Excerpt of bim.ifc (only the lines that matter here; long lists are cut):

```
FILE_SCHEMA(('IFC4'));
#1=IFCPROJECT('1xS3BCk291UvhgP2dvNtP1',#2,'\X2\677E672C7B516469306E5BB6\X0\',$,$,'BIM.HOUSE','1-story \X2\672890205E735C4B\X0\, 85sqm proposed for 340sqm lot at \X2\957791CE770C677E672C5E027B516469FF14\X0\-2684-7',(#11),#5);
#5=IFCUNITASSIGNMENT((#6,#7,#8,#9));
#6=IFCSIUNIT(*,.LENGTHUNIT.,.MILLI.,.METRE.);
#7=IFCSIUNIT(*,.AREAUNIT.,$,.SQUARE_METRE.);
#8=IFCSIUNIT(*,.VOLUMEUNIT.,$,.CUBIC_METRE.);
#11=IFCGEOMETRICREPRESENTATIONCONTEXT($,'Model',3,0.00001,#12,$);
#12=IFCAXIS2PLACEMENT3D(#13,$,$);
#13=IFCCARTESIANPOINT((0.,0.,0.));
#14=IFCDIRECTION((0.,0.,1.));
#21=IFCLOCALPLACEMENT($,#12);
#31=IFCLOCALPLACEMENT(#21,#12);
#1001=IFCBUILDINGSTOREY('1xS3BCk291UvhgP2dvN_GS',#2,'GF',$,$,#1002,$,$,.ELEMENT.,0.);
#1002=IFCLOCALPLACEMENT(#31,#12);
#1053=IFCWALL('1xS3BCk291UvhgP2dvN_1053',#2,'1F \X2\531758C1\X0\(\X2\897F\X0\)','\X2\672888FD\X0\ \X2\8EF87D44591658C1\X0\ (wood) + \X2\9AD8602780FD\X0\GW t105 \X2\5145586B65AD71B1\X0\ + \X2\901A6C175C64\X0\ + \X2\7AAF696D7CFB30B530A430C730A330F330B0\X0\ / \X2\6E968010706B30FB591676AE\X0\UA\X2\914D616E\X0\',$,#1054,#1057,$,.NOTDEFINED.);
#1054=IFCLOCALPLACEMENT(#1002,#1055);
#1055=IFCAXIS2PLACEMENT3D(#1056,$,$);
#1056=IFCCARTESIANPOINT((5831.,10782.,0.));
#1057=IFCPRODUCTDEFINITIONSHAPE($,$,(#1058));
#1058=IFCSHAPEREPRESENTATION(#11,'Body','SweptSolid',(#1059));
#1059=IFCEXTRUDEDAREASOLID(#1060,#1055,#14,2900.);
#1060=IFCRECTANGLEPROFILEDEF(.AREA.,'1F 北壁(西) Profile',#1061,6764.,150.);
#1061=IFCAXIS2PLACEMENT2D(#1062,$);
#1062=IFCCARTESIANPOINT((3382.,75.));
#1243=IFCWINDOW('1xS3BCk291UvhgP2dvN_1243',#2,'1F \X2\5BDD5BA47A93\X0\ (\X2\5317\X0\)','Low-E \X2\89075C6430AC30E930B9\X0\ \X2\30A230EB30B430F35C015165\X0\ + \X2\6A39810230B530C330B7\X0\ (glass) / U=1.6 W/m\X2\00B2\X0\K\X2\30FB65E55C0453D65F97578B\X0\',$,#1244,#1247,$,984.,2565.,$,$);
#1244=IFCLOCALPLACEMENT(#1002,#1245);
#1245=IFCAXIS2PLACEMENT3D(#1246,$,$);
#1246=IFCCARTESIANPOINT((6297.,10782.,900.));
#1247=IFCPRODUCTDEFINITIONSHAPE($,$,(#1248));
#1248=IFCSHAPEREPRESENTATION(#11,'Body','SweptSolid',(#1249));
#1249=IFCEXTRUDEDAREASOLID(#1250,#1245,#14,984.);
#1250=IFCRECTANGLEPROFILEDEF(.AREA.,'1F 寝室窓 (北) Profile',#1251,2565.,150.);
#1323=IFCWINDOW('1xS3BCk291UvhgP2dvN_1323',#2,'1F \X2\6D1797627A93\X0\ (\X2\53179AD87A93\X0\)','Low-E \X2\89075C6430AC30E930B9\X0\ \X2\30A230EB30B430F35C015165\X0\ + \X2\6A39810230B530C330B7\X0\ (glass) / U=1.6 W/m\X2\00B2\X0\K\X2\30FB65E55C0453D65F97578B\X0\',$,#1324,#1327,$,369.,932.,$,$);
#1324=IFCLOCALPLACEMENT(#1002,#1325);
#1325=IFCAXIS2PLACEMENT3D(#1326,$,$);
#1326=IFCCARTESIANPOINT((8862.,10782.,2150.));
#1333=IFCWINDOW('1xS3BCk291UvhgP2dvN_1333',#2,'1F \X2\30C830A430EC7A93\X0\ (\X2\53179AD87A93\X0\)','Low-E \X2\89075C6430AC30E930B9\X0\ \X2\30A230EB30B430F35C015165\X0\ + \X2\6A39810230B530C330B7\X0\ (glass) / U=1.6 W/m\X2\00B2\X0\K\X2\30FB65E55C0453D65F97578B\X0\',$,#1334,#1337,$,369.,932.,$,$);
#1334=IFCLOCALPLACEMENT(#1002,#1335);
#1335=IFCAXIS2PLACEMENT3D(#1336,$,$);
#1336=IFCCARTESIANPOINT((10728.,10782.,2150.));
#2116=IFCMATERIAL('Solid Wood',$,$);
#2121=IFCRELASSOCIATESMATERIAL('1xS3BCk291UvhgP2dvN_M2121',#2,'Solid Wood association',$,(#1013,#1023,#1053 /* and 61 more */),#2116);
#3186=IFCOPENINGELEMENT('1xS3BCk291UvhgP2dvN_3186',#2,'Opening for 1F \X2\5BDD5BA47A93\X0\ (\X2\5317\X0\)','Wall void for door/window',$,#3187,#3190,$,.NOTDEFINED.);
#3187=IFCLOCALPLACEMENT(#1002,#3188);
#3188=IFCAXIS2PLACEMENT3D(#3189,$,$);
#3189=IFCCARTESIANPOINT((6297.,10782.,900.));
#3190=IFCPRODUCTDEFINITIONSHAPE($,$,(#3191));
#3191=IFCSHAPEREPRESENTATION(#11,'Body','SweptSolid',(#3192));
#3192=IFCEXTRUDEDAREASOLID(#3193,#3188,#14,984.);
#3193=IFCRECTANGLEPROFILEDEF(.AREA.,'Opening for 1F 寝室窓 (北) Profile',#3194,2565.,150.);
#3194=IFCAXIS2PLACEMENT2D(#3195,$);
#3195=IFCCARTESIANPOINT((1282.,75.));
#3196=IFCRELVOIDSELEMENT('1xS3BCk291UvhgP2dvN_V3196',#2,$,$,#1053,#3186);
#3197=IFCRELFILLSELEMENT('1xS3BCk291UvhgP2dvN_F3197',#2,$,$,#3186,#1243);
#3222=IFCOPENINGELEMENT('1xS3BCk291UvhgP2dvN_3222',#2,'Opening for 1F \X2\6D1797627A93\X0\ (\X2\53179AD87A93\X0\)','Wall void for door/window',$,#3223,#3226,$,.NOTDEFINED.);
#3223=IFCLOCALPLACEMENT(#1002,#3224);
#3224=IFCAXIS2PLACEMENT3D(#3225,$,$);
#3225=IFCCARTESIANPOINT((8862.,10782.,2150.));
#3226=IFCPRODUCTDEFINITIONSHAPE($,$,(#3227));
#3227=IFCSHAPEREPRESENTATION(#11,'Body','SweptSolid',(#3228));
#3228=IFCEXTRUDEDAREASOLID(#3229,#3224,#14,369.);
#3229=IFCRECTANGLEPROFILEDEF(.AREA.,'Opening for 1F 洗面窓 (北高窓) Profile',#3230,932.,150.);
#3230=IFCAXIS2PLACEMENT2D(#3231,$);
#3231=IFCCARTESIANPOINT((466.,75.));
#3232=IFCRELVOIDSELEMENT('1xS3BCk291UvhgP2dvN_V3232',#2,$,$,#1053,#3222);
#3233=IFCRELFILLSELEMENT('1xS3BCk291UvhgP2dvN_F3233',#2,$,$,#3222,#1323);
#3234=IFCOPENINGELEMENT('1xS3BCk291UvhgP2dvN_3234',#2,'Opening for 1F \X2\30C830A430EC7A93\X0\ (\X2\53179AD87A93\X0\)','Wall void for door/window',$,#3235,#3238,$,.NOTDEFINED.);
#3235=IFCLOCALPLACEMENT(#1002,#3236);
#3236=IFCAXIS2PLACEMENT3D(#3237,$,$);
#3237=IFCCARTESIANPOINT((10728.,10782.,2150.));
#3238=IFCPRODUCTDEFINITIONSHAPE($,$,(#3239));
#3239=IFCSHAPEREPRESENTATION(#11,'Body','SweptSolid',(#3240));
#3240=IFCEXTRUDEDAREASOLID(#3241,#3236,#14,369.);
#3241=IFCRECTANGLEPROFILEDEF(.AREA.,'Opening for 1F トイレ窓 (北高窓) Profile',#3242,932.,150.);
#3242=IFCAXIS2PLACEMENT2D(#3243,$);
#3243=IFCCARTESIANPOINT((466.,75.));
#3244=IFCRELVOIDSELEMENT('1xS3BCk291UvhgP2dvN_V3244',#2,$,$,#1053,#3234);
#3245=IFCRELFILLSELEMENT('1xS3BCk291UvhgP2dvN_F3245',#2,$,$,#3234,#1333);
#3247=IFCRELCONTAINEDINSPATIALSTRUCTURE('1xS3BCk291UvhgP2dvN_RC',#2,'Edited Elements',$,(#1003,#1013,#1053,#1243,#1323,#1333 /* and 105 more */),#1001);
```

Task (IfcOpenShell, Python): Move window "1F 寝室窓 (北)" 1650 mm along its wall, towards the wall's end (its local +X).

```python
import ifcopenshell
import ifcopenshell.api.geometry
import ifcopenshell.util.placement

model = ifcopenshell.open("bim.ifc")

window = model.by_guid("1xS3BCk291UvhgP2dvN_1243")
opening = window.FillsVoids[0].RelatingOpeningElement
wall = opening.VoidsElements[0].RelatingBuildingElement

wall_matrix = ifcopenshell.util.placement.get_local_placement(wall.ObjectPlacement)
shift = wall_matrix[:3, 0] * 1650.0
before = ifcopenshell.util.placement.get_local_placement(window.ObjectPlacement)[:3, 3].copy()

# The window is not placed relative to its opening, so move both.
for product in (opening, window):
    matrix = ifcopenshell.util.placement.get_local_placement(product.ObjectPlacement)
    matrix[:3, 3] += shift
    ifcopenshell.api.geometry.edit_object_placement(model, product=product, matrix=matrix, is_si=False)

after = ifcopenshell.util.placement.get_local_placement(window.ObjectPlacement)[:3, 3]
print("window moved by", (after - before).round(3) + 0.0)

model.write("bim_updated.ifc")
```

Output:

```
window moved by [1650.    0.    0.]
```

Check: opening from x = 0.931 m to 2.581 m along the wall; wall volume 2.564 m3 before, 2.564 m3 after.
